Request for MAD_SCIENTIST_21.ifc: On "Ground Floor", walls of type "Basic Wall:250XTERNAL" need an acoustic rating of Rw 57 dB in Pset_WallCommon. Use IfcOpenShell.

First a look at what the model holds.

```python
import ifcopenshell
import ifcopenshell.util.element

model = ifcopenshell.open("MAD_SCIENTIST_21.ifc")
print(model.schema)
storey = next(s for s in model.by_type("IfcBuildingStorey") if s.Name == "Ground Floor")
walls = [e for e in ifcopenshell.util.element.get_decomposition(storey) if e.is_a("IfcWall")]
seen = {}
for e in walls:
    element_type = ifcopenshell.util.element.get_type(e)
    key = (element_type.Name if element_type != e and element_type else None, ifcopenshell.util.element.get_pset(e, "Pset_WallCommon", "AcousticRating"))
    seen[key] = seen.get(key, 0) + 1
for (name, value), count in sorted(seen.items(), key=str):
    print(count, "x", name, "|", value)
```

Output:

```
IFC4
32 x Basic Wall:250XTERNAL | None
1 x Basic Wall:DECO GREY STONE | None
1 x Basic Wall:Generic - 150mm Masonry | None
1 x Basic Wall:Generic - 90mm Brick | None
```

```python
import ifcopenshell
import ifcopenshell.api.pset
import ifcopenshell.util.element

model = ifcopenshell.open("MAD_SCIENTIST_21.ifc")

storey = next(s for s in model.by_type("IfcBuildingStorey") if s.Name == "Ground Floor")
walls = [e for e in ifcopenshell.util.element.get_decomposition(storey) if e.is_a("IfcWall")]

count = 0
for e in walls:
    element_type = ifcopenshell.util.element.get_type(e)
    if element_type in (None, e) or element_type.Name != "Basic Wall:250XTERNAL":
        continue
    # add_pset returns the element's existing set when there is one.
    pset = ifcopenshell.api.pset.add_pset(model, product=e, name="Pset_WallCommon")
    ifcopenshell.api.pset.edit_pset(model, pset=pset, properties={"AcousticRating": "Rw 57 dB"})
    count += 1

print(count, "walls updated")

model.write("MAD_SCIENTIST_21-out.ifc")
```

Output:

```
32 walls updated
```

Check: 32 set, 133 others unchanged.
